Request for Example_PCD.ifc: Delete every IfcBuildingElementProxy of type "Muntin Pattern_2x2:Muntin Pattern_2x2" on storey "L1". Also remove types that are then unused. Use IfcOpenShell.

First a look at what the model holds.

```python
import ifcopenshell
import ifcopenshell.util.element

model = ifcopenshell.open("Example_PCD.ifc")
print(model.schema)
storey = next(s for s in model.by_type("IfcBuildingStorey") if s.Name == "L1")
proxies = [e for e in ifcopenshell.util.element.get_decomposition(storey) if e.is_a("IfcBuildingElementProxy")]
seen = {}
for e in proxies:
    element_type = ifcopenshell.util.element.get_type(e)
    name = element_type.Name if element_type not in (None, e) else None
    seen[name] = seen.get(name, 0) + 1
for name, count in sorted(seen.items(), key=str):
    print(count, "x", name)
```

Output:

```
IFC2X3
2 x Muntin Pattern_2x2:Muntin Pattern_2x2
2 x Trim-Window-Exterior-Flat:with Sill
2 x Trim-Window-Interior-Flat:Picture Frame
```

```python
import ifcopenshell
import ifcopenshell.api.root
import ifcopenshell.util.element

model = ifcopenshell.open("Example_PCD.ifc")

storey = next(s for s in model.by_type("IfcBuildingStorey") if s.Name == "L1")
proxies = [e for e in ifcopenshell.util.element.get_decomposition(storey) if e.is_a("IfcBuildingElementProxy")]
targets = [e for e in proxies if (t := ifcopenshell.util.element.get_type(e)) not in (None, e) and t.Name == "Muntin Pattern_2x2:Muntin Pattern_2x2"]
types = {ifcopenshell.util.element.get_type(e) for e in targets} - {None, *targets}

for e in targets:
    ifcopenshell.api.root.remove_product(model, product=e)
print(len(targets), "removed")

unused = [t for t in types if not ifcopenshell.util.element.get_types(t)]
for t in unused:
    ifcopenshell.api.root.remove_product(model, product=t)
print(len(unused), "unused types removed")

model.write("Example_PCD_updated.ifc")
```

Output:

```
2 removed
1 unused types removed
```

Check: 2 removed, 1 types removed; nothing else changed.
